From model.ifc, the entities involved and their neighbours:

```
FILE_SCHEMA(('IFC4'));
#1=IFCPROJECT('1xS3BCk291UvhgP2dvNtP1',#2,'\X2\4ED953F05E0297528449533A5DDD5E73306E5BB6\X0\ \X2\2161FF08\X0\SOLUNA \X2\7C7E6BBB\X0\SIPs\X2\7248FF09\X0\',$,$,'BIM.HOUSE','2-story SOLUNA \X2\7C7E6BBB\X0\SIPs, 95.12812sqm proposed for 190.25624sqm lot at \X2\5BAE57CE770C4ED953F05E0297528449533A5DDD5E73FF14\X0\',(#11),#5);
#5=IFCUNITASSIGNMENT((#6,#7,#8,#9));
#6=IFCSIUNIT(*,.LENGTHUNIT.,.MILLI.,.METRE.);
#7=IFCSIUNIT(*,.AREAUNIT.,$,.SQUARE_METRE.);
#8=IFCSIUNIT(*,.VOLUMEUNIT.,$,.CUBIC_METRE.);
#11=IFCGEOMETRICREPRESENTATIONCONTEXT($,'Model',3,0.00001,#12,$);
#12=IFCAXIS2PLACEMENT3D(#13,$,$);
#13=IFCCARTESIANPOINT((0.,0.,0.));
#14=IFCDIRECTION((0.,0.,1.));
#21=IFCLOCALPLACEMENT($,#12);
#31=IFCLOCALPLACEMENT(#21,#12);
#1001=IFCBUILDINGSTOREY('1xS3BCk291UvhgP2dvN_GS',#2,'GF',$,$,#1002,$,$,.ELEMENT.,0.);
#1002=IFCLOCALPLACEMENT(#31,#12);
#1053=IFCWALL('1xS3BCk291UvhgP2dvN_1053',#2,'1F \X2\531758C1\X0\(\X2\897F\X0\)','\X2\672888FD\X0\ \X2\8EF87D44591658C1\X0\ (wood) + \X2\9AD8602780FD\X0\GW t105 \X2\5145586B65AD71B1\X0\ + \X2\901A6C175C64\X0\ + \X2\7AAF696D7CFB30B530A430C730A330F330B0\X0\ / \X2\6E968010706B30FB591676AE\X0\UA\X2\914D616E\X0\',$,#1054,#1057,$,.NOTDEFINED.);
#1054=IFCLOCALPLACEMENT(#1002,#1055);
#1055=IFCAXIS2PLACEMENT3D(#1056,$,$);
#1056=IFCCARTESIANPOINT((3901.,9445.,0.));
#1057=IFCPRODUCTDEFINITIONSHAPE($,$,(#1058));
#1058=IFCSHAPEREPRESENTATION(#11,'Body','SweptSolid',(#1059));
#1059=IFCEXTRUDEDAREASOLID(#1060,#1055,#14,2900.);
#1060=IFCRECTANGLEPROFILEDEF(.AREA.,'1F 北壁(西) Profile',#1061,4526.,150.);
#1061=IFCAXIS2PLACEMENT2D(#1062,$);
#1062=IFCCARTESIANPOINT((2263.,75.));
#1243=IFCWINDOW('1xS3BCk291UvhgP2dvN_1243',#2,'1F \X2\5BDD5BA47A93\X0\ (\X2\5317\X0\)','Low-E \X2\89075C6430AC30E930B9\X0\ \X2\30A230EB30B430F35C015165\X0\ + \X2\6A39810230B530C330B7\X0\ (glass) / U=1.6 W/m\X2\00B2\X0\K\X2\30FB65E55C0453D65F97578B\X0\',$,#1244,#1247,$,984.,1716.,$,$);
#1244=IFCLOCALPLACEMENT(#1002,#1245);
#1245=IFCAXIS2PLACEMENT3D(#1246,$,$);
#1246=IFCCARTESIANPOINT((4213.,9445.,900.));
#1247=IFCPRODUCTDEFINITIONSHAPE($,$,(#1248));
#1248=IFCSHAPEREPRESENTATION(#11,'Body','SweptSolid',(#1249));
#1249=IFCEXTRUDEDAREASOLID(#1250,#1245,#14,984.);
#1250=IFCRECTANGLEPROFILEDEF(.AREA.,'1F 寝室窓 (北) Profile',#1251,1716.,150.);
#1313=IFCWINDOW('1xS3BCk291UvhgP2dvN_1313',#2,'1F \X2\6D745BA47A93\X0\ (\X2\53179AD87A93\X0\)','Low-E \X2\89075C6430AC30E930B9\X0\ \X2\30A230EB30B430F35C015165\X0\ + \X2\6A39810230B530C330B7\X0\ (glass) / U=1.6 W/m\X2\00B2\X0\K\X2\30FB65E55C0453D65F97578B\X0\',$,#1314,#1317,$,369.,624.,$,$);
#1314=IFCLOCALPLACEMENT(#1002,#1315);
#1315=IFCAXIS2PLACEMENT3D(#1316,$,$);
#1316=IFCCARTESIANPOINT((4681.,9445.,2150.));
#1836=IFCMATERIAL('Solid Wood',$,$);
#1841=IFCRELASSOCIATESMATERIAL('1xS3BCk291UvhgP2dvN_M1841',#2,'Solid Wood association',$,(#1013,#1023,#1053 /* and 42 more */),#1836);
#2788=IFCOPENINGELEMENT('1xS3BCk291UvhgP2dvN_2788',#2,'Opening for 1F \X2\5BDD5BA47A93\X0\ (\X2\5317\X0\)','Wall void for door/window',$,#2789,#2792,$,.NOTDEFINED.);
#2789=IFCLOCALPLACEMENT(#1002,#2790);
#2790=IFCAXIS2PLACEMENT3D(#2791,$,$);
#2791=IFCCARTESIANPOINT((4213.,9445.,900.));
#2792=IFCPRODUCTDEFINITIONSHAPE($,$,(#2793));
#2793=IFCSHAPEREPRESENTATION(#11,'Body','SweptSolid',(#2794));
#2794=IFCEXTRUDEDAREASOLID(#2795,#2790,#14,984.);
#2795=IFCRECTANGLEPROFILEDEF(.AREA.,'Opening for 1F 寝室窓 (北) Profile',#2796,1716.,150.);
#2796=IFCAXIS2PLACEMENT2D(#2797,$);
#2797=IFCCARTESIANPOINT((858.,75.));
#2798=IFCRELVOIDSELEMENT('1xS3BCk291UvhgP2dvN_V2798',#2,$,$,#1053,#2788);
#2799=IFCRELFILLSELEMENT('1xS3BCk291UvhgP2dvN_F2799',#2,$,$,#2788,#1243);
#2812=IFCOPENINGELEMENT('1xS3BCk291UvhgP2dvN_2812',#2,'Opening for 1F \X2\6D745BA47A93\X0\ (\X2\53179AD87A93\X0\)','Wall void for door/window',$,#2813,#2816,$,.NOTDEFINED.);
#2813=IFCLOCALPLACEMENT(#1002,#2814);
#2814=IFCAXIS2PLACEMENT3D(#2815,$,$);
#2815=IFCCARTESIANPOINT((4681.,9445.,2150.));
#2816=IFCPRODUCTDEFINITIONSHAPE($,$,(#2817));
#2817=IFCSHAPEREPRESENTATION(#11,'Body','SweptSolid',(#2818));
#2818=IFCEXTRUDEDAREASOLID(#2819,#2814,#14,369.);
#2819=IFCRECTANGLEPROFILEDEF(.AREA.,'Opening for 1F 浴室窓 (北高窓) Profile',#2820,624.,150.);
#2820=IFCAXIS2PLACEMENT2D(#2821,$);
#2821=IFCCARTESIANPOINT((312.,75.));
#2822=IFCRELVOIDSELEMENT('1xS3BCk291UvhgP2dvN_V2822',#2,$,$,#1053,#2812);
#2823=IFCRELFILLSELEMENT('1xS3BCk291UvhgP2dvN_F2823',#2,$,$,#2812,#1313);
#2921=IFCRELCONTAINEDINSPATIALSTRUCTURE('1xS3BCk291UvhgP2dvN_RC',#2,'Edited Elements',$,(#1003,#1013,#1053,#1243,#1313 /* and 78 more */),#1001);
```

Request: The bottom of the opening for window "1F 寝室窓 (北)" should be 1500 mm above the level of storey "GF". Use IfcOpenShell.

```python
import numpy as np
import ifcopenshell
import ifcopenshell.api.geometry
import ifcopenshell.geom
import ifcopenshell.util.element
import ifcopenshell.util.placement
import ifcopenshell.util.shape
import ifcopenshell.util.unit

model = ifcopenshell.open("model.ifc")
unit_scale = ifcopenshell.util.unit.calculate_unit_scale(model)

window = model.by_id(1243)
opening = window.FillsVoids[0].RelatingOpeningElement
storey = ifcopenshell.util.element.get_container(window, ifc_class="IfcBuildingStorey")
level = ifcopenshell.util.placement.get_local_placement(storey.ObjectPlacement)[2, 3]

# The opening's origin need not be at the sill, so measure its lowest point.
shape = ifcopenshell.geom.create_shape(ifcopenshell.geom.settings(), opening)
bottom = ifcopenshell.util.shape.get_shape_bottom_elevation(shape, shape.geometry) / unit_scale
dz = level + 1500.0 - bottom

shift = np.array([0.0, 0.0, dz])
# The window is not placed relative to its opening, so move both.
for product in (opening, window):
    matrix = ifcopenshell.util.placement.get_local_placement(product.ObjectPlacement)
    matrix[:3, 3] += shift
    ifcopenshell.api.geometry.edit_object_placement(model, product=product, matrix=matrix, is_si=False)

print(f"moved by {dz * unit_scale:+.3f} m")

model.write("model_edited.ifc")
```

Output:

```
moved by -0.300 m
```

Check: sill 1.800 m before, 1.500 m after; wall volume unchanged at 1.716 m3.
